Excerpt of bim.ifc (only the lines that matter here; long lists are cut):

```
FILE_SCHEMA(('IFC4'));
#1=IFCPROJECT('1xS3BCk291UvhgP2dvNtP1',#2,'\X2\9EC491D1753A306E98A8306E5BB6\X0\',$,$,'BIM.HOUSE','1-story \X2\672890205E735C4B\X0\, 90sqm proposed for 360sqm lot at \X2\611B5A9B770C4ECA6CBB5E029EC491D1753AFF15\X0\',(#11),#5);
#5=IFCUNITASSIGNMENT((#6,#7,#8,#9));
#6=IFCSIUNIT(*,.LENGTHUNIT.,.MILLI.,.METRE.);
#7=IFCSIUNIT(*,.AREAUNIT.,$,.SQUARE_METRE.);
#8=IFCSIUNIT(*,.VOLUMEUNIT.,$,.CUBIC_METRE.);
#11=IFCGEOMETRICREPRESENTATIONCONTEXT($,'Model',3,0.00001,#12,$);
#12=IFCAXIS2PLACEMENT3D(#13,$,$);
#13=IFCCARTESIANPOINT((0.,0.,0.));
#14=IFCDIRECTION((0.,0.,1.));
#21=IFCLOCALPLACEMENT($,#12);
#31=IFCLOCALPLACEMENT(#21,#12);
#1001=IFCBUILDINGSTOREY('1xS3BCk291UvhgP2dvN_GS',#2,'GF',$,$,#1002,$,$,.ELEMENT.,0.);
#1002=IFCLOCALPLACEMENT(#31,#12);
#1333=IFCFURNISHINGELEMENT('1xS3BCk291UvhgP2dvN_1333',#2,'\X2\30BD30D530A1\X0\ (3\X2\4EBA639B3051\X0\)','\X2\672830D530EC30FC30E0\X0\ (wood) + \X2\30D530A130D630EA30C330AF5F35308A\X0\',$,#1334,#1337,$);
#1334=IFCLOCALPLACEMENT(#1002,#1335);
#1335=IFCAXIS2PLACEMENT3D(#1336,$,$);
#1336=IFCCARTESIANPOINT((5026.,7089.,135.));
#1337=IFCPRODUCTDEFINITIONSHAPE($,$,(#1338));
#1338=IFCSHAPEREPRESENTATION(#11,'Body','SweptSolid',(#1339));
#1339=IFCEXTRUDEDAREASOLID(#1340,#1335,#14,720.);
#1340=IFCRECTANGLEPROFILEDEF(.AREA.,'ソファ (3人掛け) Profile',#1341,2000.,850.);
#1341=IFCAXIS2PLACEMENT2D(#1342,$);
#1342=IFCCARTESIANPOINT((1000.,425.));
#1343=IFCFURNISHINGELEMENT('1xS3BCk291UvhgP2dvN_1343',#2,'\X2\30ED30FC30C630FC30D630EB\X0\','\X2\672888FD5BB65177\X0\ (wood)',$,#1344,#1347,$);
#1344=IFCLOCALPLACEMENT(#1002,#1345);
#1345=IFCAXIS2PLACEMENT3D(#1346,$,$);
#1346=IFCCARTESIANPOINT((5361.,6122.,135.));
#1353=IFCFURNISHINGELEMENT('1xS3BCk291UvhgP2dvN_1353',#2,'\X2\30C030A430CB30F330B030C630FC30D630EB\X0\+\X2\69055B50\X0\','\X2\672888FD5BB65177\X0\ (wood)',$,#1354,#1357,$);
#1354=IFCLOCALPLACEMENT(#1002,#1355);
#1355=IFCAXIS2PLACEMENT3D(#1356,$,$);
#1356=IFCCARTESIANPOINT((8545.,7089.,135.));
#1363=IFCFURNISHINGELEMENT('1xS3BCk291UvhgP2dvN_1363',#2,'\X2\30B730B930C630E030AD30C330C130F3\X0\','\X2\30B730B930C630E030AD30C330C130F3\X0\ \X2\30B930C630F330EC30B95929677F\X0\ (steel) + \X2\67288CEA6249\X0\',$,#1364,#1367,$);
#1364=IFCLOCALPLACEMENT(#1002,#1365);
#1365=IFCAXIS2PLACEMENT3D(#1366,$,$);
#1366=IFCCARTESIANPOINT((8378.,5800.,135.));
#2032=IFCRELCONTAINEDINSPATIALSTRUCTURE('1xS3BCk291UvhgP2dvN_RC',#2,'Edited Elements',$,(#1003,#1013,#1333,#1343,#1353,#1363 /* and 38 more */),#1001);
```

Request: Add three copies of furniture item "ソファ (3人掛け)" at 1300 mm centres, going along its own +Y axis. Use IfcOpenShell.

```python
import ifcopenshell
import ifcopenshell.api.geometry
import ifcopenshell.api.root
import ifcopenshell.util.element
import ifcopenshell.util.placement

model = ifcopenshell.open("bim.ifc")


def reuse_history(source, copy):
    """copy_class also copies each property set's owner history, people and application; keep the originals."""
    for rel in copy.IsDefinedBy:
        if rel.is_a("IfcRelDefinesByProperties") and (history := rel.RelatingPropertyDefinition.OwnerHistory):
            rel.RelatingPropertyDefinition.OwnerHistory = source.OwnerHistory
            ifcopenshell.util.element.remove_deep2(model, history)


source = model.by_guid("1xS3BCk291UvhgP2dvN_1333")
base = ifcopenshell.util.placement.get_local_placement(source.ObjectPlacement)
step = base[:3, 1] * 1300.0

for i in range(1, 4):
    copy = ifcopenshell.api.root.copy_class(model, product=source)
    copy.Representation = ifcopenshell.util.element.copy_deep(
        model, source.Representation, exclude=["IfcGeometricRepresentationContext", "IfcRepresentationMap"]
    )
    reuse_history(source, copy)
    matrix = base.copy()
    matrix[:3, 3] += i * step
    print("added at", matrix[:3, 3].round(3) + 0.0)
    ifcopenshell.api.geometry.edit_object_placement(model, product=copy, matrix=matrix, is_si=False)

model.write("bim_v2.ifc")
```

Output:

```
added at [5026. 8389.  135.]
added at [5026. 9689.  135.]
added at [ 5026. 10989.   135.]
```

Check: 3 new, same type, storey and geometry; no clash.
